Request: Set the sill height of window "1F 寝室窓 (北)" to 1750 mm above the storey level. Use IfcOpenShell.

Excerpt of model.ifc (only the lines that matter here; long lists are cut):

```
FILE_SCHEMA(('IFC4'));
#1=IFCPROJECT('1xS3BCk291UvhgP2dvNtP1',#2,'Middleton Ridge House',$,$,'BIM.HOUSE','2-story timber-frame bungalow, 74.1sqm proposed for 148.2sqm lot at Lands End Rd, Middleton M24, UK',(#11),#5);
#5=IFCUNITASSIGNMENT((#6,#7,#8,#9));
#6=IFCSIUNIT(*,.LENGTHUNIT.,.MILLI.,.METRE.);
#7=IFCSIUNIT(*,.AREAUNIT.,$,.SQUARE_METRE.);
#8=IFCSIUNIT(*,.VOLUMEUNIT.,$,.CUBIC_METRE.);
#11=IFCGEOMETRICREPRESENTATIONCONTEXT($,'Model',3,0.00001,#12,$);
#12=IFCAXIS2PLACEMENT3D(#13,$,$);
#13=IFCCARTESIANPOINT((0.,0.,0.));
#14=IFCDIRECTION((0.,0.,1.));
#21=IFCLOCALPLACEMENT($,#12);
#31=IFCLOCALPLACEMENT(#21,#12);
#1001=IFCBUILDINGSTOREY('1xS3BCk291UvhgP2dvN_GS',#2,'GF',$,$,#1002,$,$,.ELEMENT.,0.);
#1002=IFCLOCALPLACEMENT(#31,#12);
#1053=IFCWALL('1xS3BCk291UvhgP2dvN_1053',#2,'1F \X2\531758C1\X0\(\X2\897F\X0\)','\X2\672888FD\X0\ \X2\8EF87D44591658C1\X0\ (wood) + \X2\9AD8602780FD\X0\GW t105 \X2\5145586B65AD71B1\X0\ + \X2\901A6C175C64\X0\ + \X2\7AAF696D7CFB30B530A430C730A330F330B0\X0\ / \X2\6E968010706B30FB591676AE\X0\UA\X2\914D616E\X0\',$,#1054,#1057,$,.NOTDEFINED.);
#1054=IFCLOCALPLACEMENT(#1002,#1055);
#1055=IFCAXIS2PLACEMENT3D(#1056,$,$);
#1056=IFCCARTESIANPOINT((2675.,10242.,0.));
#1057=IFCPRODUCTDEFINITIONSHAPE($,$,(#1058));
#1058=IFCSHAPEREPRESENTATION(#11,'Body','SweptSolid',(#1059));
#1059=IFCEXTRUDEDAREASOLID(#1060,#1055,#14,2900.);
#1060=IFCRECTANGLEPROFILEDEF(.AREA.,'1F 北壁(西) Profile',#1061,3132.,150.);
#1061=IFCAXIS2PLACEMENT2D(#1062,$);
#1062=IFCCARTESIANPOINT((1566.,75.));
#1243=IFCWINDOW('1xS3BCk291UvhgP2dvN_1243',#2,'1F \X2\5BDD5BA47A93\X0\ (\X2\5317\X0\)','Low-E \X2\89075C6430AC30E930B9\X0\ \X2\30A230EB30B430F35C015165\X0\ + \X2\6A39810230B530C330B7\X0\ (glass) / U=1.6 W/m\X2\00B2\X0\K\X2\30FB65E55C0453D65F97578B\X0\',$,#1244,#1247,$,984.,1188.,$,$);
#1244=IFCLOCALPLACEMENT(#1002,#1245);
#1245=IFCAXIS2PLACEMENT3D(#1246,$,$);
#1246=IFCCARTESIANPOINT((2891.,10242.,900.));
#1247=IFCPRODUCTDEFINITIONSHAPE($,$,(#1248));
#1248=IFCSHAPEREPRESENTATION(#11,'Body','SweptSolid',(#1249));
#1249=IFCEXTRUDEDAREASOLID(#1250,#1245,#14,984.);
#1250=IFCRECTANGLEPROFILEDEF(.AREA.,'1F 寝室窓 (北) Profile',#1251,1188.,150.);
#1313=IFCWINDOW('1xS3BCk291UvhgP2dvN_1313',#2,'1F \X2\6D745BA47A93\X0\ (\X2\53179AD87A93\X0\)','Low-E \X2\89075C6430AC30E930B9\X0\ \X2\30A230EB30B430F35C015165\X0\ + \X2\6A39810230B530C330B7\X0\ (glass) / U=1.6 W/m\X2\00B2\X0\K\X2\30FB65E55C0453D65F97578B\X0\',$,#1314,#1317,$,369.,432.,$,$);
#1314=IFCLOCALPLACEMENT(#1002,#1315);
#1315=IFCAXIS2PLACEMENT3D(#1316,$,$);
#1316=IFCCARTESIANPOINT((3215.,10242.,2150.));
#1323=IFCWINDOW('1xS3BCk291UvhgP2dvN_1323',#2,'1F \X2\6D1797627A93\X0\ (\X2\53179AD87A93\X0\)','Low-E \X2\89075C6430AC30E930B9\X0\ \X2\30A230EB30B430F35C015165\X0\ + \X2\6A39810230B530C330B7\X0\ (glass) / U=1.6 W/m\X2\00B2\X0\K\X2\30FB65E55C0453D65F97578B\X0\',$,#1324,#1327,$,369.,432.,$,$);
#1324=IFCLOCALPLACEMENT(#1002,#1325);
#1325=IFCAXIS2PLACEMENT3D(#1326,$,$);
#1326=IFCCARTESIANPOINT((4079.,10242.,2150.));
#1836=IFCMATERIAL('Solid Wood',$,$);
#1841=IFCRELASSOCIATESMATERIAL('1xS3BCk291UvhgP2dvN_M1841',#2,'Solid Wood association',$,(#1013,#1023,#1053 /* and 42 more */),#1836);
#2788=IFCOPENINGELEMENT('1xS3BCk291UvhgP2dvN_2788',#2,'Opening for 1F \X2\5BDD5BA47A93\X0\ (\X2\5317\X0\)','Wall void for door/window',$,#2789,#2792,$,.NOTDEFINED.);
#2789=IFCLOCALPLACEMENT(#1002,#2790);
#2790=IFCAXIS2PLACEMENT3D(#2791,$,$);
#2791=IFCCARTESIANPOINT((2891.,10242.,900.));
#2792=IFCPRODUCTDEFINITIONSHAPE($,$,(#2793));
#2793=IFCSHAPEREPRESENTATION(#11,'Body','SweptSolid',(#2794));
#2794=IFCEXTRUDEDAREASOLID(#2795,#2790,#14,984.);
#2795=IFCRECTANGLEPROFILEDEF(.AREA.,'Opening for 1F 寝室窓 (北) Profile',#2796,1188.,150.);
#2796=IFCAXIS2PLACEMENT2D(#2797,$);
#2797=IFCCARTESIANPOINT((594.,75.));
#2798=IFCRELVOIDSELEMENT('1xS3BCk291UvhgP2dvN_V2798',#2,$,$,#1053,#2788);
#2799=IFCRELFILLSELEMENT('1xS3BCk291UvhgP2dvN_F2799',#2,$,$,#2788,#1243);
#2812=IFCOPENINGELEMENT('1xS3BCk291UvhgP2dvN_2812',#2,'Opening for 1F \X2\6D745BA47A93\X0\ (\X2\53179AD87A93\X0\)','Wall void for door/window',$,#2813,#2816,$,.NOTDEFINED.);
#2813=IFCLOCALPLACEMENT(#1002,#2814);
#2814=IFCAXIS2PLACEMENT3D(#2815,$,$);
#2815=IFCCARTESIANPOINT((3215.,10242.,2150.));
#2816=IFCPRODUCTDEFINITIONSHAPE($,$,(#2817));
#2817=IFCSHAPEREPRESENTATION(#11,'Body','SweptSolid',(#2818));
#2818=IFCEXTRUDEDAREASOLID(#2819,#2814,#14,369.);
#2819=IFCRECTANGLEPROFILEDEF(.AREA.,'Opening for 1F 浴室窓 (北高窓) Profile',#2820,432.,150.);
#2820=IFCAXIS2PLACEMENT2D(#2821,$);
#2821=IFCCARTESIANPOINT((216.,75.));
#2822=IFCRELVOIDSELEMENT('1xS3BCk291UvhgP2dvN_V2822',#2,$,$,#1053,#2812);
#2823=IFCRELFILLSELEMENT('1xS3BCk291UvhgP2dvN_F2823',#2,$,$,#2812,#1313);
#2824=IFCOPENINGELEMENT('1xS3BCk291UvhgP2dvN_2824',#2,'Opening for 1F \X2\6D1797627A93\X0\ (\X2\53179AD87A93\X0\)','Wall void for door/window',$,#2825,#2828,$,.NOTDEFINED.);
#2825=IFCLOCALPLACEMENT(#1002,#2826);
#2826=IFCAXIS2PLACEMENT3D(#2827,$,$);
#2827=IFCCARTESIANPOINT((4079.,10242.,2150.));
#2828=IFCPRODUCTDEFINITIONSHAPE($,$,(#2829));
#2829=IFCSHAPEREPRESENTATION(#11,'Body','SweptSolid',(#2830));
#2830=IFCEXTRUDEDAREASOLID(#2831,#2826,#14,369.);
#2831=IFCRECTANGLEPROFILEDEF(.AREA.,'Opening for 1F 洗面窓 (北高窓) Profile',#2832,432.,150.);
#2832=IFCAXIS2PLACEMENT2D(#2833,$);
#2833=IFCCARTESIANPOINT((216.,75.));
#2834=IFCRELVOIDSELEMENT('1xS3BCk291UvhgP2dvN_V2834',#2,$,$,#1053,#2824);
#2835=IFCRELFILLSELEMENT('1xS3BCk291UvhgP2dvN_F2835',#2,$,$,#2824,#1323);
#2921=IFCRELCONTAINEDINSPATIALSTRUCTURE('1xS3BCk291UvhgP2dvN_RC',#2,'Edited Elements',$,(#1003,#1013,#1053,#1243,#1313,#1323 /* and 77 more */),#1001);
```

```python
import numpy as np
import ifcopenshell
import ifcopenshell.api.geometry
import ifcopenshell.geom
import ifcopenshell.util.element
import ifcopenshell.util.placement
import ifcopenshell.util.shape
import ifcopenshell.util.unit

model = ifcopenshell.open("model.ifc")
unit_scale = ifcopenshell.util.unit.calculate_unit_scale(model)

window = model.by_guid("1xS3BCk291UvhgP2dvN_1243")
opening = window.FillsVoids[0].RelatingOpeningElement
storey = ifcopenshell.util.element.get_container(window, ifc_class="IfcBuildingStorey")
level = ifcopenshell.util.placement.get_local_placement(storey.ObjectPlacement)[2, 3]

# The opening's origin need not be at the sill, so measure its lowest point.
shape = ifcopenshell.geom.create_shape(ifcopenshell.geom.settings(), opening)
bottom = ifcopenshell.util.shape.get_shape_bottom_elevation(shape, shape.geometry) / unit_scale
dz = level + 1.75 / unit_scale - bottom

shift = np.array([0.0, 0.0, dz])
# The window is not placed relative to its opening, so move both.
for product in (opening, window):
    matrix = ifcopenshell.util.placement.get_local_placement(product.ObjectPlacement)
    matrix[:3, 3] += shift
    ifcopenshell.api.geometry.edit_object_placement(model, product=product, matrix=matrix, is_si=False)

print(f"moved by {dz * unit_scale:+.3f} m")

model.write("model_updated.ifc")
```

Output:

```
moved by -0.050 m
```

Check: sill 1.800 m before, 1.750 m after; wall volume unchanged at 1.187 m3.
